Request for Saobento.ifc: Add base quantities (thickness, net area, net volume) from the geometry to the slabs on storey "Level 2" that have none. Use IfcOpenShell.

First a look at what the model holds.

```python
import ifcopenshell
import ifcopenshell.util.element
import ifcopenshell.util.unit

model = ifcopenshell.open("Saobento.ifc")
print(model.schema)
for unit_type in ("LENGTHUNIT", "AREAUNIT", "VOLUMEUNIT"):
    print(unit_type, ifcopenshell.util.unit.calculate_unit_scale(model, unit_type))
storey = next(s for s in model.by_type("IfcBuildingStorey") if s.Name == "Level 2")
slabs = [e for e in ifcopenshell.util.element.get_decomposition(storey) if e.is_a("IfcSlab")]
for e in sorted(slabs, key=lambda e: e.id()):
    print(e.id(), e.is_a(), e.Name, list(ifcopenshell.util.element.get_psets(e, qtos_only=True)), sep=" | ")
```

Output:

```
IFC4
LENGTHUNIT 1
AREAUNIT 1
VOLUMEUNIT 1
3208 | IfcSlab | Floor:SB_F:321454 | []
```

```python
import ifcopenshell
import ifcopenshell.api.pset
import ifcopenshell.geom
import ifcopenshell.util.element
import ifcopenshell.util.shape
import ifcopenshell.util.unit

model = ifcopenshell.open("Saobento.ifc")
unit_scale = ifcopenshell.util.unit.calculate_unit_scale(model)
area_scale = ifcopenshell.util.unit.calculate_unit_scale(model, "AREAUNIT")
volume_scale = ifcopenshell.util.unit.calculate_unit_scale(model, "VOLUMEUNIT")
settings = ifcopenshell.geom.settings()

storey = next(s for s in model.by_type("IfcBuildingStorey") if s.Name == "Level 2")
slabs = [e for e in ifcopenshell.util.element.get_decomposition(storey) if e.is_a("IfcSlab")]

for e in sorted(slabs, key=lambda e: e.id()):
    if ifcopenshell.util.element.get_psets(e, qtos_only=True, should_inherit=False):
        continue
    # Geometry comes back in metres, in the element's own axes.
    shape = ifcopenshell.geom.create_shape(settings, e)
    values = {
        "Width": ifcopenshell.util.shape.get_z(shape.geometry) / unit_scale,
        "NetArea": ifcopenshell.util.shape.get_footprint_area(shape.geometry) / area_scale,
        "NetVolume": ifcopenshell.util.shape.get_volume(shape.geometry) / volume_scale,
    }
    qto = ifcopenshell.api.pset.add_qto(model, product=e, name="Qto_SlabBaseQuantities")
    ifcopenshell.api.pset.edit_qto(model, qto=qto, properties=values)
    print(e.id(), {k: round(v, 3) for k, v in values.items()})

model.write("Saobento-out.ifc")
```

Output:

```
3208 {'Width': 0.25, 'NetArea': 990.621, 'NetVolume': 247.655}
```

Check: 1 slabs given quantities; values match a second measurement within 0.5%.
